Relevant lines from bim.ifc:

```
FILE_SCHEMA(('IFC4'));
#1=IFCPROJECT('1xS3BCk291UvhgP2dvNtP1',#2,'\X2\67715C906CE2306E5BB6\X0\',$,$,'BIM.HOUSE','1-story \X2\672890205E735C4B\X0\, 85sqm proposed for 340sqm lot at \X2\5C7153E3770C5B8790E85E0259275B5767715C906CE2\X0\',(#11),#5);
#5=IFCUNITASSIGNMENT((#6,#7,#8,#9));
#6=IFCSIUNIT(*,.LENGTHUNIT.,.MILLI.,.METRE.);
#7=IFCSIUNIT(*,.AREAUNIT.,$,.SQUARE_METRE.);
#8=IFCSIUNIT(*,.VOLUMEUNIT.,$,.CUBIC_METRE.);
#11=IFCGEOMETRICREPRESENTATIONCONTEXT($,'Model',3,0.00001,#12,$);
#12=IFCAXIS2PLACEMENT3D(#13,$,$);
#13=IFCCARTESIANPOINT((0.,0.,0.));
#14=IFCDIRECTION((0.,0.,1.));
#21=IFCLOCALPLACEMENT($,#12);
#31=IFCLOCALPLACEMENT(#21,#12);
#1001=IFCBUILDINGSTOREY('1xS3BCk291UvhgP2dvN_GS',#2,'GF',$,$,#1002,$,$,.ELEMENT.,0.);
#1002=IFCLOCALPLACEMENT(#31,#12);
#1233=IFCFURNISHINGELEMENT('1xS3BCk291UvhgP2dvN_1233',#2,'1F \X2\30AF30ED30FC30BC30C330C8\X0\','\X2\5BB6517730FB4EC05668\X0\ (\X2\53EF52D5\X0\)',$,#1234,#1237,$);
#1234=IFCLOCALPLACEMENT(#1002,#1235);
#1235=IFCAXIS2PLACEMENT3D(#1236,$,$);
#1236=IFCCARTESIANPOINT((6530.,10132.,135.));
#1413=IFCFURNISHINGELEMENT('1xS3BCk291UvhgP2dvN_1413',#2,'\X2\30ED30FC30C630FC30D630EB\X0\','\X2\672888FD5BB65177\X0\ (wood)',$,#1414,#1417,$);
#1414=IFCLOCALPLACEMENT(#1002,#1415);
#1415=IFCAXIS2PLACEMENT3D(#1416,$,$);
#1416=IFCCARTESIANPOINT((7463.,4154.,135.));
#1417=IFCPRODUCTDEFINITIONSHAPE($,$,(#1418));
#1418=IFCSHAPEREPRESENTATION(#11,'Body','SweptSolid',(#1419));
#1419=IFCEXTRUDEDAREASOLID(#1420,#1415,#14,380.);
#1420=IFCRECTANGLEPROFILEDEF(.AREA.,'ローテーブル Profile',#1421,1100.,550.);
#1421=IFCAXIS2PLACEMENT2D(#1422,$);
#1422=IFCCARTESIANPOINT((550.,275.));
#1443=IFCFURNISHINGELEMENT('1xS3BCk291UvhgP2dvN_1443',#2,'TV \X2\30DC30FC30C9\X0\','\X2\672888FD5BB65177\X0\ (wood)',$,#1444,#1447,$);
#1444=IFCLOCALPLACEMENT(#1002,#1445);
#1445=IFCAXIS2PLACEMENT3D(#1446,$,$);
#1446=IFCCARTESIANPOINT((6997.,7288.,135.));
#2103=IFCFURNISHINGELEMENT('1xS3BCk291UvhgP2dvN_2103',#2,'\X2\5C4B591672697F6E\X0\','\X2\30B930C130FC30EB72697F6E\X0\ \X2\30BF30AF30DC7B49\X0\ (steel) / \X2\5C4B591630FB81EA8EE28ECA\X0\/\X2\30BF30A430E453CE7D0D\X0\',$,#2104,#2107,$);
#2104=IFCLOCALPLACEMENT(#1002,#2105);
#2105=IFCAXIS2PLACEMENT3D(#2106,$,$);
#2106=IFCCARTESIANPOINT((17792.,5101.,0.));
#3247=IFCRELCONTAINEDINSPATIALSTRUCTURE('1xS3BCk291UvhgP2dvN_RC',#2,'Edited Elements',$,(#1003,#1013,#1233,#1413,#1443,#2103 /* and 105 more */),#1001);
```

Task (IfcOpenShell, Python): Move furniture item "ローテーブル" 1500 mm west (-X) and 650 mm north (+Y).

```python
import ifcopenshell
import ifcopenshell.api.geometry
import ifcopenshell.util.placement
import ifcopenshell.util.unit

model = ifcopenshell.open("bim.ifc")
unit_scale = ifcopenshell.util.unit.calculate_unit_scale(model)

item = model.by_guid("1xS3BCk291UvhgP2dvN_1413")
matrix = ifcopenshell.util.placement.get_local_placement(item.ObjectPlacement)
matrix[0, 3] -= 1.5 / unit_scale
matrix[1, 3] += 0.65 / unit_scale
ifcopenshell.api.geometry.edit_object_placement(model, product=item, matrix=matrix, is_si=False)

print(ifcopenshell.util.placement.get_local_placement(item.ObjectPlacement).round(3) + 0.0)

model.write("bim-out.ifc")
```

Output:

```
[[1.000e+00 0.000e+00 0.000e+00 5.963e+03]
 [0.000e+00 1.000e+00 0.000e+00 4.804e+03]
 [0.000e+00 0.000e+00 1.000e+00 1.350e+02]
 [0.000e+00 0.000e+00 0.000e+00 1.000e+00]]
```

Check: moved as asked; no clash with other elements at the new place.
